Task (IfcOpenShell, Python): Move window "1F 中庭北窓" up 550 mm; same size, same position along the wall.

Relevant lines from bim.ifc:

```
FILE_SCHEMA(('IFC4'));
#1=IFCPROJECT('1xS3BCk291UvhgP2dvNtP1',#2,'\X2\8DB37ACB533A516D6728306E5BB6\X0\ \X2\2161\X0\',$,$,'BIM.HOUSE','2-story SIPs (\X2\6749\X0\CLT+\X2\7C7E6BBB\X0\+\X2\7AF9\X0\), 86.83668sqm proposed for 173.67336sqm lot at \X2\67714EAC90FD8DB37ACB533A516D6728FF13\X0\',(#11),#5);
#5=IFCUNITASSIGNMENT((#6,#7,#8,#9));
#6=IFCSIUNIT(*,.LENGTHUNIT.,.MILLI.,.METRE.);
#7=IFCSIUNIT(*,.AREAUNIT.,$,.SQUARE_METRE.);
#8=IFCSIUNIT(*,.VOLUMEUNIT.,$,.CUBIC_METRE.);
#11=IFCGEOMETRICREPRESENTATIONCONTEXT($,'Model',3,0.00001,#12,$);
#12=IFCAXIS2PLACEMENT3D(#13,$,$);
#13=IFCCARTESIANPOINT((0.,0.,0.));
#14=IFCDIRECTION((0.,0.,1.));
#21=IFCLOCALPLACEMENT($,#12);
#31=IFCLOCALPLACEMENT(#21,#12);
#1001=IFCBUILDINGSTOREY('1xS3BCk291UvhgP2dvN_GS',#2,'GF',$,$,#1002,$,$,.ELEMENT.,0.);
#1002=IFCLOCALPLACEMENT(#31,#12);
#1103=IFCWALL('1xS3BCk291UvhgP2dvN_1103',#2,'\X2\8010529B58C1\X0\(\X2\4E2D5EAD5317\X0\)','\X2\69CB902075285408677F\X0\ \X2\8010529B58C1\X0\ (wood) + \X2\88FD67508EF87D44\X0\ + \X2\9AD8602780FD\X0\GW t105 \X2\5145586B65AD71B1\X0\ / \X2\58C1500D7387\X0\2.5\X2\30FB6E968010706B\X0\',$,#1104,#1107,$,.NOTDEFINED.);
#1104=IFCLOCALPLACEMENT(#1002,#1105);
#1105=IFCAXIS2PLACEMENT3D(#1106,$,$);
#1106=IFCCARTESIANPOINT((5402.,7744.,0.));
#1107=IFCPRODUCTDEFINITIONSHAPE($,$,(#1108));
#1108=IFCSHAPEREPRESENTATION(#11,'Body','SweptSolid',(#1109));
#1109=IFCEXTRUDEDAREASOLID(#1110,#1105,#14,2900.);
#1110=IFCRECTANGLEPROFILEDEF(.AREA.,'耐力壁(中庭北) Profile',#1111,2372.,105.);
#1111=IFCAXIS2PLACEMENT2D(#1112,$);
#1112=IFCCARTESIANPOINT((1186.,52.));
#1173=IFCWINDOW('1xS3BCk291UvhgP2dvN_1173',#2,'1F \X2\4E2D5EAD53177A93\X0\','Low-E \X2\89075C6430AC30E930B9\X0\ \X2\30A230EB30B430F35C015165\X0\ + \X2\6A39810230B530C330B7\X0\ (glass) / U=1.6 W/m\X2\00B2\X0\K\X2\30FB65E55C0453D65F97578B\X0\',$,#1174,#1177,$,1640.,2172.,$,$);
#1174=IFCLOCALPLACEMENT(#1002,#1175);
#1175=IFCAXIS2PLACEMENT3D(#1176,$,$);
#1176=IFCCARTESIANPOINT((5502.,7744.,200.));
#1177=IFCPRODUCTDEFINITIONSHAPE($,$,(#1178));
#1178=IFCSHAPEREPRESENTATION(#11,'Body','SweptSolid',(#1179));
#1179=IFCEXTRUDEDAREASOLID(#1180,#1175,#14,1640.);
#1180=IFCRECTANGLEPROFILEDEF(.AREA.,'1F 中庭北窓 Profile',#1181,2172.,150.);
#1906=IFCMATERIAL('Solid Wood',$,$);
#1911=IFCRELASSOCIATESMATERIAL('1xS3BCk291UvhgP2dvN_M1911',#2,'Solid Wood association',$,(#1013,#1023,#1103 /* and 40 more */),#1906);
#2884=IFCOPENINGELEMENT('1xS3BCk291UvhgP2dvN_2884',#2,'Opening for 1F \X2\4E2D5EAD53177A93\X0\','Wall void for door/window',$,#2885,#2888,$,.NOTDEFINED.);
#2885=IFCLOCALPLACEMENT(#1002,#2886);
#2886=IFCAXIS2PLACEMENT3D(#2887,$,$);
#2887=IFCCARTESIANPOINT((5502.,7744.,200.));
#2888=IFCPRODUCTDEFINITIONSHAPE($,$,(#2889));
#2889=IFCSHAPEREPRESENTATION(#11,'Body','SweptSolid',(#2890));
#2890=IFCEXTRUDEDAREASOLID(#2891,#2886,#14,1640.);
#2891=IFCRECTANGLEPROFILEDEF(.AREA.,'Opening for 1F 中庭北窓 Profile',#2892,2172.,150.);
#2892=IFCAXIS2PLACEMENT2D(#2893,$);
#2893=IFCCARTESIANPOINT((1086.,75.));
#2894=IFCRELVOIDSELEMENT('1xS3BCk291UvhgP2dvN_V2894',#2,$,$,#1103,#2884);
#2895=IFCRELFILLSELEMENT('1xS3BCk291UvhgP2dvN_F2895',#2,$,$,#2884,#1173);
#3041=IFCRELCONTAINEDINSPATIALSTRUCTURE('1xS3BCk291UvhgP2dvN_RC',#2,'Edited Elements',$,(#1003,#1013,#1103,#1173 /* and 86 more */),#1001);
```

```python
import numpy as np
import ifcopenshell
import ifcopenshell.api.geometry
import ifcopenshell.util.placement
import ifcopenshell.util.unit

model = ifcopenshell.open("bim.ifc")
unit_scale = ifcopenshell.util.unit.calculate_unit_scale(model)

window = model.by_guid("1xS3BCk291UvhgP2dvN_1173")
opening = window.FillsVoids[0].RelatingOpeningElement
dz = 550.0

shift = np.array([0.0, 0.0, dz])
# The window is not placed relative to its opening, so move both.
for product in (opening, window):
    matrix = ifcopenshell.util.placement.get_local_placement(product.ObjectPlacement)
    matrix[:3, 3] += shift
    ifcopenshell.api.geometry.edit_object_placement(model, product=product, matrix=matrix, is_si=False)

print(f"moved by {dz * unit_scale:+.3f} m")

model.write("bim_updated.ifc")
```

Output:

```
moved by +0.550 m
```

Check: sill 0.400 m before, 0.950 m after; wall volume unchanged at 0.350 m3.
